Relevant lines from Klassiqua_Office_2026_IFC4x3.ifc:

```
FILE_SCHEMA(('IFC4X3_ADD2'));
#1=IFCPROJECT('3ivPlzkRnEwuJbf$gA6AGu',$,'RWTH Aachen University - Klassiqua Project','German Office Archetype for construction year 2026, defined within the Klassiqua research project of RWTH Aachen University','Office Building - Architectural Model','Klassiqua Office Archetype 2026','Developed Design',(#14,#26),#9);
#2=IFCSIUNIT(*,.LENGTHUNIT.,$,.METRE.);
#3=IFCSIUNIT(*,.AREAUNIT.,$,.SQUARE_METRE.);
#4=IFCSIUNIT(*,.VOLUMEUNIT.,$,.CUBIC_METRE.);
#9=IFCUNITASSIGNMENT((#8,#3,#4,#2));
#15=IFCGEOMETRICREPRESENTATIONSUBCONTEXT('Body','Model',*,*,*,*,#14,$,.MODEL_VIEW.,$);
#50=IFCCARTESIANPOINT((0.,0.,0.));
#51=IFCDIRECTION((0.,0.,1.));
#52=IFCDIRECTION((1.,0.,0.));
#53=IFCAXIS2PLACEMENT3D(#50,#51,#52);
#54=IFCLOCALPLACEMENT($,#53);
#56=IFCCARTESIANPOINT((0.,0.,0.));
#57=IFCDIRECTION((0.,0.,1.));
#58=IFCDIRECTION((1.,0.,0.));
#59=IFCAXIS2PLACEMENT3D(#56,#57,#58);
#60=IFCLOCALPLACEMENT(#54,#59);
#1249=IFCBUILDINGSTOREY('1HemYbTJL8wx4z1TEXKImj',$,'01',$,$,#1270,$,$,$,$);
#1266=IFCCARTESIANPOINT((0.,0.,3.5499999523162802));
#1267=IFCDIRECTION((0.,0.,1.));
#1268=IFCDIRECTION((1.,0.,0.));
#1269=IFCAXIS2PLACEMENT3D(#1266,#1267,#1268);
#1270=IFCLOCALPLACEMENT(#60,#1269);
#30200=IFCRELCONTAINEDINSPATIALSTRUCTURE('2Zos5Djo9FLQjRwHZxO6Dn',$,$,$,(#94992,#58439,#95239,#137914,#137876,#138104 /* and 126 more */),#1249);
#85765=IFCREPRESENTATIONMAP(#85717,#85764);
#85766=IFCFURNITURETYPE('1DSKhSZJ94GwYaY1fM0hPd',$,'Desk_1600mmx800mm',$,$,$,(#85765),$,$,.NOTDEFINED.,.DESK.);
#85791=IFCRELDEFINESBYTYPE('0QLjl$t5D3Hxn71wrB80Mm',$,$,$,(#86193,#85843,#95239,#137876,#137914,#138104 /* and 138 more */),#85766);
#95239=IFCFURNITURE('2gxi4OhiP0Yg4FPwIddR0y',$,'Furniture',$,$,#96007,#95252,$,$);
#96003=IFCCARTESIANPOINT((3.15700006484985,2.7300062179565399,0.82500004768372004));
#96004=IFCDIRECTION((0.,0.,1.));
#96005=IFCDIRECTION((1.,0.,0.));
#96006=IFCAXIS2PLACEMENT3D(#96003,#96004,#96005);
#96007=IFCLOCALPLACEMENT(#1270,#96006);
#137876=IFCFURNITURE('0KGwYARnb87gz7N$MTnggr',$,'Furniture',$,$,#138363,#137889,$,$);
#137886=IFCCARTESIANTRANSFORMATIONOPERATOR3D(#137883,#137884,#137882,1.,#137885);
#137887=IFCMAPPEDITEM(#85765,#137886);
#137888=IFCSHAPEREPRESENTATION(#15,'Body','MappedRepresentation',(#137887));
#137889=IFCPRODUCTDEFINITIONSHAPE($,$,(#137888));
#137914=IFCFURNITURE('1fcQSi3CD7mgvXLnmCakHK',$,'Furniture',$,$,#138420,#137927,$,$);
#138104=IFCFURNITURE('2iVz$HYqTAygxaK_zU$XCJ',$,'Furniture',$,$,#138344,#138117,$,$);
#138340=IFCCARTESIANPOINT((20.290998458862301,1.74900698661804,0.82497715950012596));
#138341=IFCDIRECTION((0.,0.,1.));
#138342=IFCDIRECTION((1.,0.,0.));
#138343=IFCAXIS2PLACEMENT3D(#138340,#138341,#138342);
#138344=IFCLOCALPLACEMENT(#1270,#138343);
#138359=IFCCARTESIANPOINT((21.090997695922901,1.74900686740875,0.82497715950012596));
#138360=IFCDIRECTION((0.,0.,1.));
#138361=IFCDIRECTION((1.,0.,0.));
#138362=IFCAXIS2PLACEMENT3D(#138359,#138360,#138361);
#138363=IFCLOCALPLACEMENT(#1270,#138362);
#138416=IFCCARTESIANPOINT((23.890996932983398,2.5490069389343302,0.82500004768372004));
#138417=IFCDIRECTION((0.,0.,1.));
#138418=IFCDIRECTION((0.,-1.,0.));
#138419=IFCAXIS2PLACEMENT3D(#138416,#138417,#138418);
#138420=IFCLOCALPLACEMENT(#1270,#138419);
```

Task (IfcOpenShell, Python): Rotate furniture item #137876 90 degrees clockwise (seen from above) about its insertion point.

```python
import ifcopenshell
import ifcopenshell.api.geometry
import ifcopenshell.util.placement

model = ifcopenshell.open("Klassiqua_Office_2026_IFC4x3.ifc")

item = model.by_id(137876)
matrix = ifcopenshell.util.placement.get_local_placement(item.ObjectPlacement)
matrix = matrix @ ifcopenshell.util.placement.rotation(-90, "Z")
ifcopenshell.api.geometry.edit_object_placement(model, product=item, matrix=matrix, is_si=False)

print(ifcopenshell.util.placement.get_local_placement(item.ObjectPlacement).round(3) + 0.0)

model.write("Klassiqua_Office_2026_IFC4x3_updated.ifc")
```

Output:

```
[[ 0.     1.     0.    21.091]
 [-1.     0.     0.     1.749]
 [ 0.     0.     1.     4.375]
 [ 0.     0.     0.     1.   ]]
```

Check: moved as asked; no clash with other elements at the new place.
